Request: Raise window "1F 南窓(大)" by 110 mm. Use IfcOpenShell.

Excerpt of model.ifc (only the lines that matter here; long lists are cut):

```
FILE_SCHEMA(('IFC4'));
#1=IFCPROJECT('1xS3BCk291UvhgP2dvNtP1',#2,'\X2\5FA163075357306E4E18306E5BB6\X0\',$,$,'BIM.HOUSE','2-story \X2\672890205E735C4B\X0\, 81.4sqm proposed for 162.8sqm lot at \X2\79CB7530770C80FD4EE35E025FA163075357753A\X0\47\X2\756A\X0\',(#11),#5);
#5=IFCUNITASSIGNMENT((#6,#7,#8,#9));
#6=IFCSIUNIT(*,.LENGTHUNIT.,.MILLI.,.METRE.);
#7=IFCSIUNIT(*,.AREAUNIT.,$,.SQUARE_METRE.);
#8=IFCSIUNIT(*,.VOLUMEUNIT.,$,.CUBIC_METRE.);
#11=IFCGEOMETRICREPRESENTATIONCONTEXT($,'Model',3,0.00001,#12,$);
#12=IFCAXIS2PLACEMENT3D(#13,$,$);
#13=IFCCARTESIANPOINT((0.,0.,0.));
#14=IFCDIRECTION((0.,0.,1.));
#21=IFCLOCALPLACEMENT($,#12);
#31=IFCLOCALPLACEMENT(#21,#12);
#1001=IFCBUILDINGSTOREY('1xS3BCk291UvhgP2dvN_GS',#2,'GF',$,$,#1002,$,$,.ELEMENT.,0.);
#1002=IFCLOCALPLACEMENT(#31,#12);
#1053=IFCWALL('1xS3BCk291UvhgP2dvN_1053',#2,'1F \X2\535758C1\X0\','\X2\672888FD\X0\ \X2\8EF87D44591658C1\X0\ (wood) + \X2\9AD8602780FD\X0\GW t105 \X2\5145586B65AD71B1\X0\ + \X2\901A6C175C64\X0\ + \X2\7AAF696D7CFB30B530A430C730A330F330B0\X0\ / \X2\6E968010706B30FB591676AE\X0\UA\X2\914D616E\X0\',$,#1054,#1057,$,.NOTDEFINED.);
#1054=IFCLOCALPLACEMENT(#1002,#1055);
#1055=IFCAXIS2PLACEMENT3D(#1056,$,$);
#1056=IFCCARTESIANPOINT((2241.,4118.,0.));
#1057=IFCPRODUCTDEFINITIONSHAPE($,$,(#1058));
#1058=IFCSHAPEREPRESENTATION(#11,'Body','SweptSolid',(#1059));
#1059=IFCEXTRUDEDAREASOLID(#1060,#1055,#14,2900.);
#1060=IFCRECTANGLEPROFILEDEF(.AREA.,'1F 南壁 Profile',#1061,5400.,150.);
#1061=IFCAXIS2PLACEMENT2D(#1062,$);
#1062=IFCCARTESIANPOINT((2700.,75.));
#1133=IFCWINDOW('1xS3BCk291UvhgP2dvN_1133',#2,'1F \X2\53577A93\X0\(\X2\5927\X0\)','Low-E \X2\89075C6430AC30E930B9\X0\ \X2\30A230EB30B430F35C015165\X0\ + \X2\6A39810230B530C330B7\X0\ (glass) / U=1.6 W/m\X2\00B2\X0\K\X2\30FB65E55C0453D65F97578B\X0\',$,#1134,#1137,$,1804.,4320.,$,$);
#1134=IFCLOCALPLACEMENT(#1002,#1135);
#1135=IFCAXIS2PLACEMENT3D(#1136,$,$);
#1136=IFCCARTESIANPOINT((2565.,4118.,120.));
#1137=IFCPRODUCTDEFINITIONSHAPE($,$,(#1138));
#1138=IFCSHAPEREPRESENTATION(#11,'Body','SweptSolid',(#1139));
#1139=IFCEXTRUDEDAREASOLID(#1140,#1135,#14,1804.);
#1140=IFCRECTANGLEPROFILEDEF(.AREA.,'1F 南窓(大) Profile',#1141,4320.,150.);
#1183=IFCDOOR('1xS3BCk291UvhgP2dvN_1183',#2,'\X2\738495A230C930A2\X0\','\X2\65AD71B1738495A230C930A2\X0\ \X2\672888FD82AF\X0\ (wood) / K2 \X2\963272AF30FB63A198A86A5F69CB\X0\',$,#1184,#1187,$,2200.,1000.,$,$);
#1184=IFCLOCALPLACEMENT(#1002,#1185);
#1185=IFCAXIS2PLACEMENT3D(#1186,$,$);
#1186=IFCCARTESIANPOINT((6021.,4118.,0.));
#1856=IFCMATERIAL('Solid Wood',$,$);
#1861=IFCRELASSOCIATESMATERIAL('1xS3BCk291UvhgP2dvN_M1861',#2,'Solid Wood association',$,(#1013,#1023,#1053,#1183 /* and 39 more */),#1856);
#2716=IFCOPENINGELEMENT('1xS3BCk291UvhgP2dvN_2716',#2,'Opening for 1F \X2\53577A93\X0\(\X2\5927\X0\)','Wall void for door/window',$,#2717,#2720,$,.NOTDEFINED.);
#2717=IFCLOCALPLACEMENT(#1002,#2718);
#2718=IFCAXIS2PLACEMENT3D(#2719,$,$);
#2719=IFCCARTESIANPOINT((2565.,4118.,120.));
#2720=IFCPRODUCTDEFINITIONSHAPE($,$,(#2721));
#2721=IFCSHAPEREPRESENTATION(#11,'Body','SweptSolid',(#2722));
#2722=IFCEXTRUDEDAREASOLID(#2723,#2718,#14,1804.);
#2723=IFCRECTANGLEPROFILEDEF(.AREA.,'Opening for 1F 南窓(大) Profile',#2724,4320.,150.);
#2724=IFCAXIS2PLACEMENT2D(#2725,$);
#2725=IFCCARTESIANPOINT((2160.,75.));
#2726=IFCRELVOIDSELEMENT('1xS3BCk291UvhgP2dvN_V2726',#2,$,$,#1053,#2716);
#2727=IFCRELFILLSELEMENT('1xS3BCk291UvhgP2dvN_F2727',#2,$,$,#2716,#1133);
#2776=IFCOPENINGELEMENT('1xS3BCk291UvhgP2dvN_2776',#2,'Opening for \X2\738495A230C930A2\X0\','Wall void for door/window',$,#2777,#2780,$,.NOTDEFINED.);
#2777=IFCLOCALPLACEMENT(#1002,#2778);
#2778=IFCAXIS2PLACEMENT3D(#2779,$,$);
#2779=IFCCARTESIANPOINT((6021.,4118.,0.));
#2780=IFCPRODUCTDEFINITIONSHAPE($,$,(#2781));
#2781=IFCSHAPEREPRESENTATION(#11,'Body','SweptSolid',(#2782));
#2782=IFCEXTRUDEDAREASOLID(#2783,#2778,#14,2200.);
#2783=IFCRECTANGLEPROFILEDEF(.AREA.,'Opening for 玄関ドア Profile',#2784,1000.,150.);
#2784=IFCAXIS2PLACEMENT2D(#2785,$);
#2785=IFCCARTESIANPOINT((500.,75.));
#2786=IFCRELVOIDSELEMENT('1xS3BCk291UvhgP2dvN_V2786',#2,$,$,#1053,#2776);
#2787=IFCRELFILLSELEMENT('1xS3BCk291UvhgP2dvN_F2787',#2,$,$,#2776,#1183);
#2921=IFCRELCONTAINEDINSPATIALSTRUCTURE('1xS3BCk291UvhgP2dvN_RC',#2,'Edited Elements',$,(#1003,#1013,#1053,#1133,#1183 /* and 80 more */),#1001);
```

```python
import numpy as np
import ifcopenshell
import ifcopenshell.api.geometry
import ifcopenshell.util.placement
import ifcopenshell.util.unit

model = ifcopenshell.open("model.ifc")
unit_scale = ifcopenshell.util.unit.calculate_unit_scale(model)

window = model.by_id(1133)
opening = window.FillsVoids[0].RelatingOpeningElement
dz = 0.11 / unit_scale

shift = np.array([0.0, 0.0, dz])
# The window is not placed relative to its opening, so move both.
for product in (opening, window):
    matrix = ifcopenshell.util.placement.get_local_placement(product.ObjectPlacement)
    matrix[:3, 3] += shift
    ifcopenshell.api.geometry.edit_object_placement(model, product=product, matrix=matrix, is_si=False)

print(f"moved by {dz * unit_scale:+.3f} m")

model.write("model-out.ifc")
```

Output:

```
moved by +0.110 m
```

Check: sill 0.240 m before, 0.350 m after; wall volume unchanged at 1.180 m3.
